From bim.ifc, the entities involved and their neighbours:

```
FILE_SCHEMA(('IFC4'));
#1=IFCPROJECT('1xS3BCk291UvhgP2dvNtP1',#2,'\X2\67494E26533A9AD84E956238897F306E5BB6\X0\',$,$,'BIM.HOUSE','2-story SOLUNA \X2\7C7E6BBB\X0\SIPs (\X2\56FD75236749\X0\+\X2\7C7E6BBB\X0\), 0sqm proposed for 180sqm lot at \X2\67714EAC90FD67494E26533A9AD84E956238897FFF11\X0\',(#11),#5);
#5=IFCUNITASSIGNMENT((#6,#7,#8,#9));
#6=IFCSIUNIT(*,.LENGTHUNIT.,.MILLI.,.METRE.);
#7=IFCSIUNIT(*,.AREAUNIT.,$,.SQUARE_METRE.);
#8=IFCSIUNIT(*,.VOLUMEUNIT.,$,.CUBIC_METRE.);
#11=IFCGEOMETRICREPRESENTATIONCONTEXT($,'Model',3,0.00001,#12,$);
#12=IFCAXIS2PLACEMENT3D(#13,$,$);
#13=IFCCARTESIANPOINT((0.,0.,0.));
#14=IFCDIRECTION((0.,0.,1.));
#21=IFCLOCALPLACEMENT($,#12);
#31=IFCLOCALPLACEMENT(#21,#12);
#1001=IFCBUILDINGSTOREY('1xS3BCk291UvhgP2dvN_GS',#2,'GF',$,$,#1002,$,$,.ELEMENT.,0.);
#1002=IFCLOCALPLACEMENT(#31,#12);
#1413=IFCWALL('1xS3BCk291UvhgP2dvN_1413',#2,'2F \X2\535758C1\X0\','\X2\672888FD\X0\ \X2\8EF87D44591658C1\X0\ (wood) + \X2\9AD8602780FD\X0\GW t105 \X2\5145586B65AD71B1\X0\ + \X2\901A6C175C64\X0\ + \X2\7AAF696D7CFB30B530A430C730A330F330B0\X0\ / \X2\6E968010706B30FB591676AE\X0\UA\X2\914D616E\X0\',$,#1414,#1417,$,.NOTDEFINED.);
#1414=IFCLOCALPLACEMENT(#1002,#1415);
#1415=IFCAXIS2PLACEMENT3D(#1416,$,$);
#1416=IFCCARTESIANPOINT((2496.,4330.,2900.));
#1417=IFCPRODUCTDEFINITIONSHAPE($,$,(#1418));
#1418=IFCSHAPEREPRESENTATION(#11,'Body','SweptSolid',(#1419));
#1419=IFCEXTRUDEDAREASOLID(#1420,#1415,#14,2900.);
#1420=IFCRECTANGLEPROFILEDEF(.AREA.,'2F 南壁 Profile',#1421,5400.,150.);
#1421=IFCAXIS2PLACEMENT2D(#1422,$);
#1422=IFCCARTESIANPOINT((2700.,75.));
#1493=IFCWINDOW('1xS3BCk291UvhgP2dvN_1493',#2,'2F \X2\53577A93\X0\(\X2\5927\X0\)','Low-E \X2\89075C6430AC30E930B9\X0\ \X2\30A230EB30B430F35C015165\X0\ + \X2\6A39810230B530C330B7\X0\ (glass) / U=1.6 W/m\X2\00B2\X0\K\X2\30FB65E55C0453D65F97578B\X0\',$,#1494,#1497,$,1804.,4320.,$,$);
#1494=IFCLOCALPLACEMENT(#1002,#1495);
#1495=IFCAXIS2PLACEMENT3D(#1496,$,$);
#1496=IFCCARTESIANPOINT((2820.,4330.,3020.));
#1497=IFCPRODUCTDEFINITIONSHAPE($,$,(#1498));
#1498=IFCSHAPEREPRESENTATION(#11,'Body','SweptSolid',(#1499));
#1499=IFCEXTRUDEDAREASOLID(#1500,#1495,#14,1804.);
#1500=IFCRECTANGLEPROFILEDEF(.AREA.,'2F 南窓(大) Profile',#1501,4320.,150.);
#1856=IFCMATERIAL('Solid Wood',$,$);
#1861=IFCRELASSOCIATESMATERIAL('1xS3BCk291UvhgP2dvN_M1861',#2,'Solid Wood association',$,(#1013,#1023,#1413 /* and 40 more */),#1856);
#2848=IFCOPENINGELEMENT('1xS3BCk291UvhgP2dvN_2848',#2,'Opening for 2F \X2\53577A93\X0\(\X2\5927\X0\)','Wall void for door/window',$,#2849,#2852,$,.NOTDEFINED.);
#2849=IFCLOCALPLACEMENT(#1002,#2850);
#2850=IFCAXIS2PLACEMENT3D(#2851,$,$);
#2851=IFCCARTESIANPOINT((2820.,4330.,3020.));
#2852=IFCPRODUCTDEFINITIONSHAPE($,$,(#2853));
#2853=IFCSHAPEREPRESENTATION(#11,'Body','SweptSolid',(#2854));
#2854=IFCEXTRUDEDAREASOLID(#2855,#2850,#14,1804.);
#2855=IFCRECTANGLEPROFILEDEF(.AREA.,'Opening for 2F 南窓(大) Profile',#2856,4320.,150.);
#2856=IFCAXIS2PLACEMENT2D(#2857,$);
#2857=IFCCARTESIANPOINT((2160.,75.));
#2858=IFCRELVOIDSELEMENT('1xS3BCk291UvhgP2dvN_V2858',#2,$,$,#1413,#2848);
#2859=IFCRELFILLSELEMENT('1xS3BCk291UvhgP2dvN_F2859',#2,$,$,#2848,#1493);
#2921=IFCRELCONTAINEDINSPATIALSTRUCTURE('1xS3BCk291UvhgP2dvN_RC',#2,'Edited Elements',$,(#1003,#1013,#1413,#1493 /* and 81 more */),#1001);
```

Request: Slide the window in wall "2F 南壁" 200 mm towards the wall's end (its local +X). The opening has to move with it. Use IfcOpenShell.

```python
import ifcopenshell
import ifcopenshell.api.geometry
import ifcopenshell.util.placement
import ifcopenshell.util.unit

model = ifcopenshell.open("bim.ifc")
unit_scale = ifcopenshell.util.unit.calculate_unit_scale(model)

window = model.by_guid("1xS3BCk291UvhgP2dvN_1493")
opening = window.FillsVoids[0].RelatingOpeningElement
wall = opening.VoidsElements[0].RelatingBuildingElement

wall_matrix = ifcopenshell.util.placement.get_local_placement(wall.ObjectPlacement)
shift = wall_matrix[:3, 0] * 0.2 / unit_scale
before = ifcopenshell.util.placement.get_local_placement(window.ObjectPlacement)[:3, 3].copy()

# The window is not placed relative to its opening, so move both.
for product in (opening, window):
    matrix = ifcopenshell.util.placement.get_local_placement(product.ObjectPlacement)
    matrix[:3, 3] += shift
    ifcopenshell.api.geometry.edit_object_placement(model, product=product, matrix=matrix, is_si=False)

after = ifcopenshell.util.placement.get_local_placement(window.ObjectPlacement)[:3, 3]
print("window moved by", (after - before).round(3) + 0.0)

model.write("bim-out.ifc")
```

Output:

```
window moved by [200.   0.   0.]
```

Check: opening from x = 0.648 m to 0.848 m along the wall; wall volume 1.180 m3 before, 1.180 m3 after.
